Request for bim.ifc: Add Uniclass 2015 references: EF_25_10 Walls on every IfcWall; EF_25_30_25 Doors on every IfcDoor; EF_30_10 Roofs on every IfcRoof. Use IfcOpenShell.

First a look at what the model holds.

```python
import ifcopenshell

model = ifcopenshell.open("bim.ifc")
print(model.schema)
print("classifications:", [c.Name for c in model.by_type("IfcClassification")])
for ifc_class in ("IfcDoor", "IfcRoof", "IfcStair", "IfcWall", "IfcWindow"):
    print(ifc_class, len(model.by_type(ifc_class)))
```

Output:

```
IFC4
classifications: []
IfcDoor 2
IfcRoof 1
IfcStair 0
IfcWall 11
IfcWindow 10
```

```python
import ifcopenshell
import ifcopenshell.api.classification

model = ifcopenshell.open("bim.ifc")

system = ifcopenshell.api.classification.add_classification(model, classification="Uniclass 2015")

codes = {
    "IfcWall": ("EF_25_10", "Walls"),
    "IfcDoor": ("EF_25_30_25", "Doors"),
    "IfcRoof": ("EF_30_10", "Roofs"),
}
for ifc_class, (code, name) in codes.items():
    products = model.by_type(ifc_class)
    ifcopenshell.api.classification.add_reference(
        model, products=products, classification=system, identification=code, name=name
    )
    print(code, len(products))

model.write("bim-out.ifc")
```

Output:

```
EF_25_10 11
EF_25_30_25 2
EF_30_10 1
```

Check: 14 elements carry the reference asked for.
